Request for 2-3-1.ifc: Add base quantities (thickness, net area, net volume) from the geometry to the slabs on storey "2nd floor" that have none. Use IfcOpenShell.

First a look at what the model holds.

```python
import ifcopenshell
import ifcopenshell.util.element
import ifcopenshell.util.unit

model = ifcopenshell.open("2-3-1.ifc")
print(model.schema)
for unit_type in ("LENGTHUNIT", "AREAUNIT", "VOLUMEUNIT"):
    print(unit_type, ifcopenshell.util.unit.calculate_unit_scale(model, unit_type))
storey = next(s for s in model.by_type("IfcBuildingStorey") if s.Name == "2nd floor")
slabs = [e for e in ifcopenshell.util.element.get_decomposition(storey) if e.is_a("IfcSlab")]
for e in sorted(slabs, key=lambda e: e.id()):
    print(e.id(), e.is_a(), e.Name, list(ifcopenshell.util.element.get_psets(e, qtos_only=True)), sep=" | ")
```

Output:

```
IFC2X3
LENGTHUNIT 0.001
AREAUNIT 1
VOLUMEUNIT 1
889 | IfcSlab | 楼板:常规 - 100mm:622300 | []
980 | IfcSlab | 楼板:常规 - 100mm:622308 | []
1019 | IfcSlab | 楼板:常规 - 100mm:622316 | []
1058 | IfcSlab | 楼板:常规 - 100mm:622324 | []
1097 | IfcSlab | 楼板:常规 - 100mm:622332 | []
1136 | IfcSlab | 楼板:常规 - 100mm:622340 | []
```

```python
import ifcopenshell
import ifcopenshell.api.pset
import ifcopenshell.geom
import ifcopenshell.util.element
import ifcopenshell.util.shape
import ifcopenshell.util.unit

model = ifcopenshell.open("2-3-1.ifc")
unit_scale = ifcopenshell.util.unit.calculate_unit_scale(model)
area_scale = ifcopenshell.util.unit.calculate_unit_scale(model, "AREAUNIT")
volume_scale = ifcopenshell.util.unit.calculate_unit_scale(model, "VOLUMEUNIT")
settings = ifcopenshell.geom.settings()

storey = next(s for s in model.by_type("IfcBuildingStorey") if s.Name == "2nd floor")
slabs = [e for e in ifcopenshell.util.element.get_decomposition(storey) if e.is_a("IfcSlab")]

for e in sorted(slabs, key=lambda e: e.id()):
    if ifcopenshell.util.element.get_psets(e, qtos_only=True, should_inherit=False):
        continue
    # Geometry comes back in metres, in the element's own axes.
    shape = ifcopenshell.geom.create_shape(settings, e)
    values = {
        "Width": ifcopenshell.util.shape.get_z(shape.geometry) / unit_scale,
        "NetArea": ifcopenshell.util.shape.get_footprint_area(shape.geometry) / area_scale,
        "NetVolume": ifcopenshell.util.shape.get_volume(shape.geometry) / volume_scale,
    }
    qto = ifcopenshell.api.pset.add_qto(model, product=e, name="BaseQuantities")
    ifcopenshell.api.pset.edit_qto(model, qto=qto, properties=values)
    print(e.id(), {k: round(v, 3) for k, v in values.items()})

model.write("2-3-1_v2.ifc")
```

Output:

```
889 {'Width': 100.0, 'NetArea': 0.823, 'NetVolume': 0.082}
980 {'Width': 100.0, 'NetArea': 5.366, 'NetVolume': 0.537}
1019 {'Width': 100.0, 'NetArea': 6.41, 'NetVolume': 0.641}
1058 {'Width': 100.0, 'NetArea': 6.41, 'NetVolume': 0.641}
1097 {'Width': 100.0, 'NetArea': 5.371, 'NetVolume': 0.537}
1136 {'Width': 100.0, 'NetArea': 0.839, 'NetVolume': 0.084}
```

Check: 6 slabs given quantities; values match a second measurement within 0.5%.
